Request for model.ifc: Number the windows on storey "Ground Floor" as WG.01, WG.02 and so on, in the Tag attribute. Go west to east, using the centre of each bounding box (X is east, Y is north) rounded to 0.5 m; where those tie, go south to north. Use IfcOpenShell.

First a look at what the model holds.

```python
import ifcopenshell
import ifcopenshell.util.element
import ifcopenshell.util.placement

model = ifcopenshell.open("model.ifc")
print(model.schema)
storey = next(s for s in model.by_type("IfcBuildingStorey") if s.Name == "Ground Floor")
windows = [e for e in ifcopenshell.util.element.get_decomposition(storey) if e.is_a("IfcWindow")]
for e in sorted(windows, key=lambda e: e.id()):
    origin = ifcopenshell.util.placement.get_local_placement(e.ObjectPlacement)[:3, 3]
    print(e.id(), e.Tag, e.Name, origin.round(2) + 0.0, sep=" | ")
```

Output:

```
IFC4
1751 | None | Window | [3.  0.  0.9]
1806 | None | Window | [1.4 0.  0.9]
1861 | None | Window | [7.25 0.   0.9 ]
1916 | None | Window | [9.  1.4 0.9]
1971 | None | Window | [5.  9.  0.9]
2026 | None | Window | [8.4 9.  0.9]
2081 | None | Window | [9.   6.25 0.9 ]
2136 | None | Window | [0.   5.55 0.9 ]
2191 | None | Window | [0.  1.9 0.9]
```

```python
import ifcopenshell
import ifcopenshell.geom
import ifcopenshell.util.element
import ifcopenshell.util.shape

model = ifcopenshell.open("model.ifc")
settings = ifcopenshell.geom.settings()
settings.set("use-world-coords", True)


def centre(element):
    shape = ifcopenshell.geom.create_shape(settings, element)
    return ifcopenshell.util.shape.get_bbox_centroid(shape.geometry)


storey = next(s for s in model.by_type("IfcBuildingStorey") if s.Name == "Ground Floor")
windows = [e for e in ifcopenshell.util.element.get_decomposition(storey) if e.is_a("IfcWindow")]

# Insertion points can sit at a corner or the storey origin, so sort by the geometry (in metres).
centres = {e: centre(e) for e in windows}
windows.sort(key=lambda e: (round(centres[e][0] / 0.5), centres[e][1]))

for i, e in enumerate(windows, start=1):
    number = f"WG.{i:02d}"
    e.Tag = number
    print(e.id(), number)

model.write("model_v2.ifc")
```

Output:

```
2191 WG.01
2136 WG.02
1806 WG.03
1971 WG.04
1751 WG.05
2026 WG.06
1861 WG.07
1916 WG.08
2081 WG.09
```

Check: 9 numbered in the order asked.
